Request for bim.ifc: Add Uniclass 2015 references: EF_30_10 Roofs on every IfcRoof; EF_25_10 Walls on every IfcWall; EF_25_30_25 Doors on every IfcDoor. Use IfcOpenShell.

First a look at what the model holds.

```python
import ifcopenshell

model = ifcopenshell.open("bim.ifc")
print(model.schema)
print("classifications:", [c.Name for c in model.by_type("IfcClassification")])
for ifc_class in ("IfcDoor", "IfcRoof", "IfcStair", "IfcWall", "IfcWindow"):
    print(ifc_class, len(model.by_type(ifc_class)))
```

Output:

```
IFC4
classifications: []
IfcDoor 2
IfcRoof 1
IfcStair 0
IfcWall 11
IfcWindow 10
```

```python
import ifcopenshell
import ifcopenshell.api.classification

model = ifcopenshell.open("bim.ifc")

system = ifcopenshell.api.classification.add_classification(model, classification="Uniclass 2015")

codes = {
    "IfcRoof": ("EF_30_10", "Roofs"),
    "IfcWall": ("EF_25_10", "Walls"),
    "IfcDoor": ("EF_25_30_25", "Doors"),
}
for ifc_class, (code, name) in codes.items():
    products = model.by_type(ifc_class)
    ifcopenshell.api.classification.add_reference(
        model, products=products, classification=system, identification=code, name=name
    )
    print(code, len(products))

model.write("bim_edited.ifc")
```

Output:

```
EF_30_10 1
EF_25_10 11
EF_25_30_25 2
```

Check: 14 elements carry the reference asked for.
